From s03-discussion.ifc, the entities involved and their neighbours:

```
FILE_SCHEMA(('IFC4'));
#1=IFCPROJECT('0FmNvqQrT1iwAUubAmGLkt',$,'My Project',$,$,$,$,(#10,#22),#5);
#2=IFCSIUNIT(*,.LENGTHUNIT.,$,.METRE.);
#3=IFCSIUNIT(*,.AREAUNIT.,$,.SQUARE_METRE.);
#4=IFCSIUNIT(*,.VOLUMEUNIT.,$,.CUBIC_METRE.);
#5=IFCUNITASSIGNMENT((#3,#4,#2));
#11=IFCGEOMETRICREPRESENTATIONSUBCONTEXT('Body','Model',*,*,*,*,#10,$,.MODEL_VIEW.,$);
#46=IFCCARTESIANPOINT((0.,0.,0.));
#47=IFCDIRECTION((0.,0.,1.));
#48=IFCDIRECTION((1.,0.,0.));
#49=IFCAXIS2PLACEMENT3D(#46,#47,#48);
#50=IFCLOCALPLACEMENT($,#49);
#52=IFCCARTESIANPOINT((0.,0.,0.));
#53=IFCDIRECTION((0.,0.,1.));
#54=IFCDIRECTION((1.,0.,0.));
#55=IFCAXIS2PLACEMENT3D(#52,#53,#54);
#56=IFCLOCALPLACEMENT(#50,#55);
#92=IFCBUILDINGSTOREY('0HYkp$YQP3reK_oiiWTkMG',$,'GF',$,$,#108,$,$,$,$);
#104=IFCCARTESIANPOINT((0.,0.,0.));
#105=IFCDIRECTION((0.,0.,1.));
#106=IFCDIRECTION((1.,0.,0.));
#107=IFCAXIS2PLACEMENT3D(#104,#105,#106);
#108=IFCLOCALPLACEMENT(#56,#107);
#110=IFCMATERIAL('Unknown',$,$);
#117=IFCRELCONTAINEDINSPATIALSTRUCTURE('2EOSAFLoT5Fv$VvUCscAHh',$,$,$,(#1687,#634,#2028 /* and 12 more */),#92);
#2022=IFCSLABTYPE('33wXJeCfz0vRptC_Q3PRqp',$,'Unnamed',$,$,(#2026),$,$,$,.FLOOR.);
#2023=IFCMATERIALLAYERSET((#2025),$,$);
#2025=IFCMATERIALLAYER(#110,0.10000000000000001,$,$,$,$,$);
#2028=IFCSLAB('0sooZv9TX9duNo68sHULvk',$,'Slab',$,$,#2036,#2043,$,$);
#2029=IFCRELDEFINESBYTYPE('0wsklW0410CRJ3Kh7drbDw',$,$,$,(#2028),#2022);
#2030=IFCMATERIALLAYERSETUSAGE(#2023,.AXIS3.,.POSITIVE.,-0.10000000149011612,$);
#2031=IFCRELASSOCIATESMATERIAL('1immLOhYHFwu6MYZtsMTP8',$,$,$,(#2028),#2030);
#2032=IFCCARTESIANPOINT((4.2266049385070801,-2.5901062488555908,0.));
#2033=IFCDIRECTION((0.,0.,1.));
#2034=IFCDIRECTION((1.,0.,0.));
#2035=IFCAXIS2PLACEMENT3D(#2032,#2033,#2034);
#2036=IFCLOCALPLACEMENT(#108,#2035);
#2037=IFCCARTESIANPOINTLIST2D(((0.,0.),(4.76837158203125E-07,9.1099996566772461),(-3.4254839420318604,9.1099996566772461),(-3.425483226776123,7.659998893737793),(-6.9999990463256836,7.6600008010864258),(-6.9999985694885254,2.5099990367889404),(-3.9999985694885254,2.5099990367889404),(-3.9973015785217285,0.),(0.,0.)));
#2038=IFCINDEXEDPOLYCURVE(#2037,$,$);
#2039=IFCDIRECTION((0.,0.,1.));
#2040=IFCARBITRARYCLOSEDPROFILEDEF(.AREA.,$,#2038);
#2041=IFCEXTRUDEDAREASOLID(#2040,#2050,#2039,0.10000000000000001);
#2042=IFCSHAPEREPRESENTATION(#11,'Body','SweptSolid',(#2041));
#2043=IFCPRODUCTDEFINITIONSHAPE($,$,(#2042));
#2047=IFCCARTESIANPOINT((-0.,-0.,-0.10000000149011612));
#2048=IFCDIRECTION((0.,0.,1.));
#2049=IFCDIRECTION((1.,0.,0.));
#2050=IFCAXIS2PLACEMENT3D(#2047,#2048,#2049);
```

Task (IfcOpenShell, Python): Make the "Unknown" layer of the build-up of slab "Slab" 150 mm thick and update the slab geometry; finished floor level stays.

```python
import ifcopenshell
import ifcopenshell.util.element
import ifcopenshell.util.representation

model = ifcopenshell.open("s03-discussion.ifc")

layer_set = model.by_id(2023)
layer = next(l for l in layer_set.MaterialLayers if l.Material and l.Material.Name == "Unknown")
change = 0.15 - layer.LayerThickness
layer.LayerThickness += change

# Geometry does not follow the layer set by itself.
slabs = [e for e in ifcopenshell.util.element.get_elements_by_material(model, layer_set) if e.is_a("IfcSlab")]
for slab in sorted(slabs, key=lambda e: e.id()):
    body = ifcopenshell.util.representation.get_representation(slab, "Model", "Body")
    solid = body.Items[0]
    old_depth = solid.Depth
    solid.Depth += change
    # Extruded upwards: lower the start of the extrusion so the top stays.
    x, y, z = solid.Position.Location.Coordinates
    solid.Position.Location = model.createIfcCartesianPoint((x, y, z - change))
    print(slab.id(), f"{old_depth:g} -> {solid.Depth:g}")

# The layers are counted up from the underside, which has moved.
for usage in {ifcopenshell.util.element.get_material(slab) for slab in slabs}:
    usage.OffsetFromReferenceLine -= change

model.write("s03-discussion_v2.ifc")
```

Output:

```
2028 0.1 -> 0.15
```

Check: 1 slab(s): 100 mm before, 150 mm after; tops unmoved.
